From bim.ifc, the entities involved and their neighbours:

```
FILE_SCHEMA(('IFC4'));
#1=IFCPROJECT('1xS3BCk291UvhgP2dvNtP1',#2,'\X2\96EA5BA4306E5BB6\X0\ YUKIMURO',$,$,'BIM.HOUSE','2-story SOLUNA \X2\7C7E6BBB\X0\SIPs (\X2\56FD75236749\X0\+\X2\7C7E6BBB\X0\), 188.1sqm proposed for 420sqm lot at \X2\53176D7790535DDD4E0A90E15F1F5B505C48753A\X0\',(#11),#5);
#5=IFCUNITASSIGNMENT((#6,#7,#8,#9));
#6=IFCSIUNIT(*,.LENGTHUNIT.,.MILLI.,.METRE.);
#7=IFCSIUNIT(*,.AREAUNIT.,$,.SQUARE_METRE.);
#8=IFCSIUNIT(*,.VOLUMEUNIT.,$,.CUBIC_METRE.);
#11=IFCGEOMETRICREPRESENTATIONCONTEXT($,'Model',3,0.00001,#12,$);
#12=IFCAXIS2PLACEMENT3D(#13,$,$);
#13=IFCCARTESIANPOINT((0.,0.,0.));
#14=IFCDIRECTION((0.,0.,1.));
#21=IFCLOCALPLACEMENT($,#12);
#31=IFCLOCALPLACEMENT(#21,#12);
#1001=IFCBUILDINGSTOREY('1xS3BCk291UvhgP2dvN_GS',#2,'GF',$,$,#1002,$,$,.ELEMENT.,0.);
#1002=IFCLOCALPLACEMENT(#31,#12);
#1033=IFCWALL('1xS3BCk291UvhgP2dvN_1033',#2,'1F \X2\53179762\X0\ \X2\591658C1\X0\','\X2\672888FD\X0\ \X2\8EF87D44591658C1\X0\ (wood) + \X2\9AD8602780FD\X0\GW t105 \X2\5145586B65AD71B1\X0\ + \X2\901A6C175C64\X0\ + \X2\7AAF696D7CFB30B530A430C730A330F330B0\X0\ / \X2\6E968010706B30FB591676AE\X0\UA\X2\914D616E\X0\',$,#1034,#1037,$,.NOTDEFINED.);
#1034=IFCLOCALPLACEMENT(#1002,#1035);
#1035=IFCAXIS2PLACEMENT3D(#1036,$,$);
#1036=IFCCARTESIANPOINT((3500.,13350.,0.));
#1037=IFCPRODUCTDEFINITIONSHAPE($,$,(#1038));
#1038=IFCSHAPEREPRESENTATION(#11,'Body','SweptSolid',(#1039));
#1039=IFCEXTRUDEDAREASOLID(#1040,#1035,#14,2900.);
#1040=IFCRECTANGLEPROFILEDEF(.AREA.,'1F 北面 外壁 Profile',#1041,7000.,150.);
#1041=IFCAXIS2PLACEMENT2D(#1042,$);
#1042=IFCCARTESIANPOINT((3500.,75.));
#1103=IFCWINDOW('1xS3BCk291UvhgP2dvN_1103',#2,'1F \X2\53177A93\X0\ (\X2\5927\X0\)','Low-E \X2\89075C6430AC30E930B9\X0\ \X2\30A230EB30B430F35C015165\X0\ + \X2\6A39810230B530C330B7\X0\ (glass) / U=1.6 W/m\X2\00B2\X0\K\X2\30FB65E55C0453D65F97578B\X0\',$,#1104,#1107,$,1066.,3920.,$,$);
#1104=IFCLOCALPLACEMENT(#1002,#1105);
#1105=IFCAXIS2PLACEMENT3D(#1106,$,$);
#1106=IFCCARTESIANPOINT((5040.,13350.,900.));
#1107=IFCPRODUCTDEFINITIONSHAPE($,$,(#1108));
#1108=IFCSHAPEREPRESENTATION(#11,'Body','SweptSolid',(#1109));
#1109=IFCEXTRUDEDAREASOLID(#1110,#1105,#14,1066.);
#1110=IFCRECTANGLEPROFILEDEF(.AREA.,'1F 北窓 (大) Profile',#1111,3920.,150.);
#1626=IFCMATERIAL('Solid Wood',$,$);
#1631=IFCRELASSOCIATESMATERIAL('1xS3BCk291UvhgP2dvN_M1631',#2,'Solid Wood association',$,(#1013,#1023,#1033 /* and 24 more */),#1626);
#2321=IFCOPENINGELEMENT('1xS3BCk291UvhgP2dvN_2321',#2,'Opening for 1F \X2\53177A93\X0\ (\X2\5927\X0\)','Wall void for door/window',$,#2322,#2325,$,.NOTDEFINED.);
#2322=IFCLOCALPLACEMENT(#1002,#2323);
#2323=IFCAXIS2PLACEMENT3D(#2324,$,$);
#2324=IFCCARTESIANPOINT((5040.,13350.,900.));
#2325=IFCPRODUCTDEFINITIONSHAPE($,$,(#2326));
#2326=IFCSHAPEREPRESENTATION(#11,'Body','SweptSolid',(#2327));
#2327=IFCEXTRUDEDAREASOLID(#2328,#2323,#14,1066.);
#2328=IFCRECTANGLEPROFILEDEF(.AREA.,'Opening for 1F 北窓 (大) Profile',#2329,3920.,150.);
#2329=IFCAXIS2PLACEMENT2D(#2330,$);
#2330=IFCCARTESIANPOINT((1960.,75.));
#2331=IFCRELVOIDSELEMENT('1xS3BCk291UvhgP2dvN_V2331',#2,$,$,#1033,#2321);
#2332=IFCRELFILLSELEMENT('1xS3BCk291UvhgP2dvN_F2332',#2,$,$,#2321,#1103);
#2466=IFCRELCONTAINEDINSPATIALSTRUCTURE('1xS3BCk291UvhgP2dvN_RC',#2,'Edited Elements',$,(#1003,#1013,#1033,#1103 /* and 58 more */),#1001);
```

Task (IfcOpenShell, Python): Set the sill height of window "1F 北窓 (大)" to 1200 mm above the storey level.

```python
import numpy as np
import ifcopenshell
import ifcopenshell.api.geometry
import ifcopenshell.geom
import ifcopenshell.util.element
import ifcopenshell.util.placement
import ifcopenshell.util.shape
import ifcopenshell.util.unit

model = ifcopenshell.open("bim.ifc")
unit_scale = ifcopenshell.util.unit.calculate_unit_scale(model)

window = model.by_guid("1xS3BCk291UvhgP2dvN_1103")
opening = window.FillsVoids[0].RelatingOpeningElement
storey = ifcopenshell.util.element.get_container(window, ifc_class="IfcBuildingStorey")
level = ifcopenshell.util.placement.get_local_placement(storey.ObjectPlacement)[2, 3]

# The opening's origin need not be at the sill, so measure its lowest point.
shape = ifcopenshell.geom.create_shape(ifcopenshell.geom.settings(), opening)
bottom = ifcopenshell.util.shape.get_shape_bottom_elevation(shape, shape.geometry) / unit_scale
dz = level + 1200.0 - bottom

shift = np.array([0.0, 0.0, dz])
# The window is not placed relative to its opening, so move both.
for product in (opening, window):
    matrix = ifcopenshell.util.placement.get_local_placement(product.ObjectPlacement)
    matrix[:3, 3] += shift
    ifcopenshell.api.geometry.edit_object_placement(model, product=product, matrix=matrix, is_si=False)

print(f"moved by {dz * unit_scale:+.3f} m")

model.write("bim_v2.ifc")
```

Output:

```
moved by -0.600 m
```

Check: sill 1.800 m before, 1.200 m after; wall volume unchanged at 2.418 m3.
